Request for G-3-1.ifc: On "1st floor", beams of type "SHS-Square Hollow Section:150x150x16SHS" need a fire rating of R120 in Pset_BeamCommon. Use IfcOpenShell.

First a look at what the model holds.

```python
import ifcopenshell
import ifcopenshell.util.element

model = ifcopenshell.open("G-3-1.ifc")
print(model.schema)
storey = next(s for s in model.by_type("IfcBuildingStorey") if s.Name == "1st floor")
beams = [e for e in ifcopenshell.util.element.get_decomposition(storey) if e.is_a("IfcBeam")]
seen = {}
for e in beams:
    element_type = ifcopenshell.util.element.get_type(e)
    key = (element_type.Name if element_type != e and element_type else None, ifcopenshell.util.element.get_pset(e, "Pset_BeamCommon", "FireRating"))
    seen[key] = seen.get(key, 0) + 1
for (name, value), count in sorted(seen.items(), key=str):
    print(count, "x", name, "|", value)
```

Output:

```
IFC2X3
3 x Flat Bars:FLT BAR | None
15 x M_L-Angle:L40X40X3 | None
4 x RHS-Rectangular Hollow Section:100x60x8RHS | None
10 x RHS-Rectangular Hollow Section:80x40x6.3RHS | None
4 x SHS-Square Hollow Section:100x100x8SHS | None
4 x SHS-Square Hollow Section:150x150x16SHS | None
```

```python
import ifcopenshell
import ifcopenshell.api.pset
import ifcopenshell.util.element

model = ifcopenshell.open("G-3-1.ifc")

storey = next(s for s in model.by_type("IfcBuildingStorey") if s.Name == "1st floor")
beams = [e for e in ifcopenshell.util.element.get_decomposition(storey) if e.is_a("IfcBeam")]

count = 0
for e in beams:
    element_type = ifcopenshell.util.element.get_type(e)
    if element_type in (None, e) or element_type.Name != "SHS-Square Hollow Section:150x150x16SHS":
        continue
    # add_pset returns the element's existing set when there is one.
    pset = ifcopenshell.api.pset.add_pset(model, product=e, name="Pset_BeamCommon")
    ifcopenshell.api.pset.edit_pset(model, pset=pset, properties={"FireRating": "R120"})
    count += 1

print(count, "beams updated")

model.write("G-3-1_v2.ifc")
```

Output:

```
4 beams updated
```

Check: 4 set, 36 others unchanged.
